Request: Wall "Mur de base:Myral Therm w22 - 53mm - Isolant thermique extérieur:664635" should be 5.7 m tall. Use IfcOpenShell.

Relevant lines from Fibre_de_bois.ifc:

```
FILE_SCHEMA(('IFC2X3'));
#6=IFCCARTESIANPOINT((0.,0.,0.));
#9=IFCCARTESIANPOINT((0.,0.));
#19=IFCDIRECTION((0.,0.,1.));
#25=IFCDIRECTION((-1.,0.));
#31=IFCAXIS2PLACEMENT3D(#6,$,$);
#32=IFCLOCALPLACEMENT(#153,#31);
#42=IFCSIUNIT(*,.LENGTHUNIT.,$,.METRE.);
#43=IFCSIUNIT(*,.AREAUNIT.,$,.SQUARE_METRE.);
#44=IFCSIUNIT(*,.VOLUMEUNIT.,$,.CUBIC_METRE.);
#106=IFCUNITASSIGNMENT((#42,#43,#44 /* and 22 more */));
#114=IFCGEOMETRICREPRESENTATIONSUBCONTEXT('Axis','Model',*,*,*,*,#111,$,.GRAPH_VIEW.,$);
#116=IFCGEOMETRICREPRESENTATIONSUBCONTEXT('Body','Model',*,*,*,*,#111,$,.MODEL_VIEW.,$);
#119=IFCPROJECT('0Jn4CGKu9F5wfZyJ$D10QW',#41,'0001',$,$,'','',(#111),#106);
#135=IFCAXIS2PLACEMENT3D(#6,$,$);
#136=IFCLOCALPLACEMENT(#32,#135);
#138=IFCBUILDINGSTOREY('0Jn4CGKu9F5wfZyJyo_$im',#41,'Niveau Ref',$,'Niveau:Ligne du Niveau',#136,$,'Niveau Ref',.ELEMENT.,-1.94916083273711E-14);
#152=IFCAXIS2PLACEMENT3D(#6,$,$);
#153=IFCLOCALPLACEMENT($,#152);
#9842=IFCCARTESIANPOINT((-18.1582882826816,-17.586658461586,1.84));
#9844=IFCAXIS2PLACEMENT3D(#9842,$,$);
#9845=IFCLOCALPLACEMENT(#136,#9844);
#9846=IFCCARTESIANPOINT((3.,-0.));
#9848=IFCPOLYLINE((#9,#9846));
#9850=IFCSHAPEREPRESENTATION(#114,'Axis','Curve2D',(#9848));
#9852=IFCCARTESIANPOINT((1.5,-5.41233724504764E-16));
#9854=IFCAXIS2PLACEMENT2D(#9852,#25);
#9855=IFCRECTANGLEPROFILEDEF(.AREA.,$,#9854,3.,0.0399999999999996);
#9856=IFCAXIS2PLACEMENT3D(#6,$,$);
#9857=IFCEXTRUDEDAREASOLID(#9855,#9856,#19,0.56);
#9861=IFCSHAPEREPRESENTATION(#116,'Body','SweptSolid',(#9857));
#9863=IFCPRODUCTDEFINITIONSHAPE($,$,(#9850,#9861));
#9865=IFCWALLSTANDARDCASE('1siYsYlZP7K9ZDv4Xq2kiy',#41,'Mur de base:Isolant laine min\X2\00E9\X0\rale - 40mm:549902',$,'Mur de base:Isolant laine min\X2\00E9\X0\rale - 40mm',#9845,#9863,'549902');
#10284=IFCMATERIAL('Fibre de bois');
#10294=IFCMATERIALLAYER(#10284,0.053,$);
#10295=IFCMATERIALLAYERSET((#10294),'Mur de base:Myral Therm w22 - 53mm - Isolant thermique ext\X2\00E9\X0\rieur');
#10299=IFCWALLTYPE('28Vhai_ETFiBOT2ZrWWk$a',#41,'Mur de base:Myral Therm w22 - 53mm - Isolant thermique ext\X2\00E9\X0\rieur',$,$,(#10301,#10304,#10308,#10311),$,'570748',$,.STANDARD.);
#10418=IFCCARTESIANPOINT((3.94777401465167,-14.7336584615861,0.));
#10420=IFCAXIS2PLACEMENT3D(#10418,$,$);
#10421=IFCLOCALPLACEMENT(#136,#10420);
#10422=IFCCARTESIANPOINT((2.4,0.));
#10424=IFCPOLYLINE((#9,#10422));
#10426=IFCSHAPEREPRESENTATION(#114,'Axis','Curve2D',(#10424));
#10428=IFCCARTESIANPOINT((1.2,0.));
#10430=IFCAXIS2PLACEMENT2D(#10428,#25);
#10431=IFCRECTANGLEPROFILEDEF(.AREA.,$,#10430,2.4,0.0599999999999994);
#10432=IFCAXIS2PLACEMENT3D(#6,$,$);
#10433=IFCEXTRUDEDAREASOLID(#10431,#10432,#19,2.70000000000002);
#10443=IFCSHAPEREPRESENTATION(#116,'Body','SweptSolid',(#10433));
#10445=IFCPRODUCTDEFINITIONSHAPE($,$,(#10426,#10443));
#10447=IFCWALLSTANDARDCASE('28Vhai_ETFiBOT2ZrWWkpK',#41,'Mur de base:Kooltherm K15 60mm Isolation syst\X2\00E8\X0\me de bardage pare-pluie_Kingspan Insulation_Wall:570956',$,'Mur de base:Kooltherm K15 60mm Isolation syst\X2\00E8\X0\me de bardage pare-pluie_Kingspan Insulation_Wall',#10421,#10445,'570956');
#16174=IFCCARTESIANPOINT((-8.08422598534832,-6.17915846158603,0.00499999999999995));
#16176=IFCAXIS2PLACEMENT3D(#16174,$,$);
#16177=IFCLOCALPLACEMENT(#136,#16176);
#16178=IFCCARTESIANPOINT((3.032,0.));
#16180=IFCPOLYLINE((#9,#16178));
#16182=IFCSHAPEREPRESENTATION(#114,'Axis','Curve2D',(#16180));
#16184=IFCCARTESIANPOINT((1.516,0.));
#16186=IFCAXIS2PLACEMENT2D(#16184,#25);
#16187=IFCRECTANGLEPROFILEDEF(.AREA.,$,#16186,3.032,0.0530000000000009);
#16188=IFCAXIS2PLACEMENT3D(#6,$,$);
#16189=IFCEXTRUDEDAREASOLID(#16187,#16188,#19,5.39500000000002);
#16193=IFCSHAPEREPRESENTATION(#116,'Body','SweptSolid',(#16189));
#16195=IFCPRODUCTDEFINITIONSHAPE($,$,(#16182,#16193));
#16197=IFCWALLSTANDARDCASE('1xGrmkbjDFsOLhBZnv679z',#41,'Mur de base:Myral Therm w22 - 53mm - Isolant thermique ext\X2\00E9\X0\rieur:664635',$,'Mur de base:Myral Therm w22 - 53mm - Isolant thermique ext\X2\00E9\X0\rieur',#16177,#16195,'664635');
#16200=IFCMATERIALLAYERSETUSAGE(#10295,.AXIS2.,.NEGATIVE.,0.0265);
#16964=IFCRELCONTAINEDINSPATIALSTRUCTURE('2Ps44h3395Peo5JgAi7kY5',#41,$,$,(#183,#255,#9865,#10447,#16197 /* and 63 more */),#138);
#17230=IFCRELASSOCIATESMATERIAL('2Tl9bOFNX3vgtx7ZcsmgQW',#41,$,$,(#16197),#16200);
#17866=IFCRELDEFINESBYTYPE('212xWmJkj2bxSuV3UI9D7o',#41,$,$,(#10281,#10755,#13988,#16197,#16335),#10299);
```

```python
import ifcopenshell
import ifcopenshell.geom
import ifcopenshell.util.representation
import ifcopenshell.util.shape
import ifcopenshell.util.unit

model = ifcopenshell.open("Fibre_de_bois.ifc")
unit_scale = ifcopenshell.util.unit.calculate_unit_scale(model)
settings = ifcopenshell.geom.settings()


def volume(element):
    """Net volume in cubic metres, openings subtracted."""
    shape = ifcopenshell.geom.create_shape(settings, element)
    return ifcopenshell.util.shape.get_volume(shape.geometry)


wall = model.by_guid("1xGrmkbjDFsOLhBZnv679z")
before = volume(wall)

body = ifcopenshell.util.representation.get_representation(wall, "Model", "Body")
solid = body.Items[0]
old_height = solid.Depth
solid.Depth = 5.7 / unit_scale
after = volume(wall)

print(f"height {old_height:g} -> {solid.Depth:g}, volume {before:.3f} -> {after:.3f} m3")

model.write("Fibre_de_bois-out.ifc")
```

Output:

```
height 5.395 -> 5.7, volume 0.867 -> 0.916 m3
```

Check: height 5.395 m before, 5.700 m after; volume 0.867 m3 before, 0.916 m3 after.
